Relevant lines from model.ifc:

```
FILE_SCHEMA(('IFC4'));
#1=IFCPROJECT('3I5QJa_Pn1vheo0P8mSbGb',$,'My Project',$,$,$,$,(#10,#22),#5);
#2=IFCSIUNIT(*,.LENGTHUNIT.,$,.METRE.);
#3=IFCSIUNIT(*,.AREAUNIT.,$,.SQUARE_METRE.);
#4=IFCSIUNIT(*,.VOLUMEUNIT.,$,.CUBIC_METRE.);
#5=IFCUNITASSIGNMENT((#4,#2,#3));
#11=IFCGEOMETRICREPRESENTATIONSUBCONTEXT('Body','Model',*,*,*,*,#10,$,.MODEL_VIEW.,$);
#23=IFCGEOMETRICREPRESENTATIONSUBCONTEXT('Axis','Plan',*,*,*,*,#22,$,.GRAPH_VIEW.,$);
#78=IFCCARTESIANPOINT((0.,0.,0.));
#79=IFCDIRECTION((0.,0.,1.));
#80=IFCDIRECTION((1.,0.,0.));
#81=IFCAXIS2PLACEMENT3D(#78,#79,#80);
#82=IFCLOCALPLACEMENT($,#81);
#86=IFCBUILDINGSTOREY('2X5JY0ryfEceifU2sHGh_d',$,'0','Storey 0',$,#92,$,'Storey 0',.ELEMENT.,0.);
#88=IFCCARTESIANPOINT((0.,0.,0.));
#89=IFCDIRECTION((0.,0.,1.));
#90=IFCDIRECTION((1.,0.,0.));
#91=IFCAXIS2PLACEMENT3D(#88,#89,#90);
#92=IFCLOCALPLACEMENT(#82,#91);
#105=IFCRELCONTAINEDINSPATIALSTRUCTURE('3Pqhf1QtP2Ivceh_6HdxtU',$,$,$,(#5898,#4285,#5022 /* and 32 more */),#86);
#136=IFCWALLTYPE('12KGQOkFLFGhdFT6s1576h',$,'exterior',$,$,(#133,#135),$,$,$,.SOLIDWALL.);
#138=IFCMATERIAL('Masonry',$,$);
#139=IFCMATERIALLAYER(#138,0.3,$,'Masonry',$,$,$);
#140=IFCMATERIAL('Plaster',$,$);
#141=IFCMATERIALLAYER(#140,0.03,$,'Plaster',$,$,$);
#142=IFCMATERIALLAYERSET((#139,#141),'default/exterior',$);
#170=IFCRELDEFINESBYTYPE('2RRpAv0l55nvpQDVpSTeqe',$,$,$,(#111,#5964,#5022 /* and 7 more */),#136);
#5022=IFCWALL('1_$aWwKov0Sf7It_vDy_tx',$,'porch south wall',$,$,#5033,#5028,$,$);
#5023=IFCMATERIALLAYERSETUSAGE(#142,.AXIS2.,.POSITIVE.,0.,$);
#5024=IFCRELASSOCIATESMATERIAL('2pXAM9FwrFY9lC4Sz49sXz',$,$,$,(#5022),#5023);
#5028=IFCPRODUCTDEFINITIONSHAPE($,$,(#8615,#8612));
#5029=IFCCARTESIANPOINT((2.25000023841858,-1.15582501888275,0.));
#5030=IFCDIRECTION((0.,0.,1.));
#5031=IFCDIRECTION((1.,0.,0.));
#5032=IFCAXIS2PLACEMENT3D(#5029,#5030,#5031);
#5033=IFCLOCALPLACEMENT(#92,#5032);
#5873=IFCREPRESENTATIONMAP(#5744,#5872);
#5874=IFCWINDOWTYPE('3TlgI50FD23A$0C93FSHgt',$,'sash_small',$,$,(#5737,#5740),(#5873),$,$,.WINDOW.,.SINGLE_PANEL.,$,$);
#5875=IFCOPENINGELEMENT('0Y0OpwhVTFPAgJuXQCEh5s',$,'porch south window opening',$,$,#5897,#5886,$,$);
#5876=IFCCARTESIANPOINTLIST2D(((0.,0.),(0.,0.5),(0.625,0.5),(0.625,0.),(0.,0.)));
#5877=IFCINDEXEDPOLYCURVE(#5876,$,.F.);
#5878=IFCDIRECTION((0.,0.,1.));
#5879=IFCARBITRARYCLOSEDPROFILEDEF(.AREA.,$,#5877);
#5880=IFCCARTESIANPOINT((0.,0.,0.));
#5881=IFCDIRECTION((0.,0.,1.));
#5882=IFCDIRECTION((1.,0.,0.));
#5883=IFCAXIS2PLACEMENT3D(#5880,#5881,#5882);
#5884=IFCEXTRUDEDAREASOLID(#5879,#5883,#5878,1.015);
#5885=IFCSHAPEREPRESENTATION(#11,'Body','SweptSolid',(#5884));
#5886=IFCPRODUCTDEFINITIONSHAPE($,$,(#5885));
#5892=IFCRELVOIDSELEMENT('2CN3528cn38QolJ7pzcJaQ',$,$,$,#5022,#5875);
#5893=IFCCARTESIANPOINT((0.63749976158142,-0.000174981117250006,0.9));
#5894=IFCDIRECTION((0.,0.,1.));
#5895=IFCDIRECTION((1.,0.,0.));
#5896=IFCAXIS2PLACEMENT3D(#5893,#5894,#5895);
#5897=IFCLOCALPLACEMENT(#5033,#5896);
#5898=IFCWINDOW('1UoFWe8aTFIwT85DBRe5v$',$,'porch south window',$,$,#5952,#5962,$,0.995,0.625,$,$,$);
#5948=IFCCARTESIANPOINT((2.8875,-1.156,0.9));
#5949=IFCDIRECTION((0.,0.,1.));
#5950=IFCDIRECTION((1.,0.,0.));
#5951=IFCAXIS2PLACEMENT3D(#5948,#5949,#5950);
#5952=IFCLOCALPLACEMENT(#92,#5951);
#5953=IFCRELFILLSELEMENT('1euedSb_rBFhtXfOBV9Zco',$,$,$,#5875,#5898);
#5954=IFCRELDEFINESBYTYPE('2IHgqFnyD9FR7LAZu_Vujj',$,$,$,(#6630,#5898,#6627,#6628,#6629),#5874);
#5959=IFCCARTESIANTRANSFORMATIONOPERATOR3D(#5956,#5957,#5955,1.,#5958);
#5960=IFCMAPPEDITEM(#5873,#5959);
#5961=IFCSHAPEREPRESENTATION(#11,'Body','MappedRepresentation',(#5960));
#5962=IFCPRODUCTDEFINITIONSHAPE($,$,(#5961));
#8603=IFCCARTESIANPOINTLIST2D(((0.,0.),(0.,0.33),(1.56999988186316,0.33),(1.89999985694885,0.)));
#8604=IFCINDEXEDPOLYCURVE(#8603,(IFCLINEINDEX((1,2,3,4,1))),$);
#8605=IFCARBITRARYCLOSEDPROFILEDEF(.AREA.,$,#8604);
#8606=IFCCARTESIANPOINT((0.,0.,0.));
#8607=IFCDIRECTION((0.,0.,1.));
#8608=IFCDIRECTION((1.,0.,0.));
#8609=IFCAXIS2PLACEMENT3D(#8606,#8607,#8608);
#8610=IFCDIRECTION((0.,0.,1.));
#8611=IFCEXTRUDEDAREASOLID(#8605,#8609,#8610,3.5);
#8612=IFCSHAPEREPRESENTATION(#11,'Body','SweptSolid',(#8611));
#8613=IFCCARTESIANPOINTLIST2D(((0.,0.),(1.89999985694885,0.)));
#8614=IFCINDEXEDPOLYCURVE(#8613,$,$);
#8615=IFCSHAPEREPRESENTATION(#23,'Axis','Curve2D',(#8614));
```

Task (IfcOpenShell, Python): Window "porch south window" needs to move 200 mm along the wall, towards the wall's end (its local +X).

```python
import ifcopenshell
import ifcopenshell.api.geometry
import ifcopenshell.util.placement

model = ifcopenshell.open("model.ifc")

window = model.by_id(5898)
opening = window.FillsVoids[0].RelatingOpeningElement
wall = opening.VoidsElements[0].RelatingBuildingElement

wall_matrix = ifcopenshell.util.placement.get_local_placement(wall.ObjectPlacement)
shift = wall_matrix[:3, 0] * 0.2
before = ifcopenshell.util.placement.get_local_placement(window.ObjectPlacement)[:3, 3].copy()

# The window is not placed relative to its opening, so move both.
for product in (opening, window):
    matrix = ifcopenshell.util.placement.get_local_placement(product.ObjectPlacement)
    matrix[:3, 3] += shift
    ifcopenshell.api.geometry.edit_object_placement(model, product=product, matrix=matrix, is_si=False)

after = ifcopenshell.util.placement.get_local_placement(window.ObjectPlacement)[:3, 3]
print("window moved by", (after - before).round(3) + 0.0)

model.write("model_edited.ifc")
```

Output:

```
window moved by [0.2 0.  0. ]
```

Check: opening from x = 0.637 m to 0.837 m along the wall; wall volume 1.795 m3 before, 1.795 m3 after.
